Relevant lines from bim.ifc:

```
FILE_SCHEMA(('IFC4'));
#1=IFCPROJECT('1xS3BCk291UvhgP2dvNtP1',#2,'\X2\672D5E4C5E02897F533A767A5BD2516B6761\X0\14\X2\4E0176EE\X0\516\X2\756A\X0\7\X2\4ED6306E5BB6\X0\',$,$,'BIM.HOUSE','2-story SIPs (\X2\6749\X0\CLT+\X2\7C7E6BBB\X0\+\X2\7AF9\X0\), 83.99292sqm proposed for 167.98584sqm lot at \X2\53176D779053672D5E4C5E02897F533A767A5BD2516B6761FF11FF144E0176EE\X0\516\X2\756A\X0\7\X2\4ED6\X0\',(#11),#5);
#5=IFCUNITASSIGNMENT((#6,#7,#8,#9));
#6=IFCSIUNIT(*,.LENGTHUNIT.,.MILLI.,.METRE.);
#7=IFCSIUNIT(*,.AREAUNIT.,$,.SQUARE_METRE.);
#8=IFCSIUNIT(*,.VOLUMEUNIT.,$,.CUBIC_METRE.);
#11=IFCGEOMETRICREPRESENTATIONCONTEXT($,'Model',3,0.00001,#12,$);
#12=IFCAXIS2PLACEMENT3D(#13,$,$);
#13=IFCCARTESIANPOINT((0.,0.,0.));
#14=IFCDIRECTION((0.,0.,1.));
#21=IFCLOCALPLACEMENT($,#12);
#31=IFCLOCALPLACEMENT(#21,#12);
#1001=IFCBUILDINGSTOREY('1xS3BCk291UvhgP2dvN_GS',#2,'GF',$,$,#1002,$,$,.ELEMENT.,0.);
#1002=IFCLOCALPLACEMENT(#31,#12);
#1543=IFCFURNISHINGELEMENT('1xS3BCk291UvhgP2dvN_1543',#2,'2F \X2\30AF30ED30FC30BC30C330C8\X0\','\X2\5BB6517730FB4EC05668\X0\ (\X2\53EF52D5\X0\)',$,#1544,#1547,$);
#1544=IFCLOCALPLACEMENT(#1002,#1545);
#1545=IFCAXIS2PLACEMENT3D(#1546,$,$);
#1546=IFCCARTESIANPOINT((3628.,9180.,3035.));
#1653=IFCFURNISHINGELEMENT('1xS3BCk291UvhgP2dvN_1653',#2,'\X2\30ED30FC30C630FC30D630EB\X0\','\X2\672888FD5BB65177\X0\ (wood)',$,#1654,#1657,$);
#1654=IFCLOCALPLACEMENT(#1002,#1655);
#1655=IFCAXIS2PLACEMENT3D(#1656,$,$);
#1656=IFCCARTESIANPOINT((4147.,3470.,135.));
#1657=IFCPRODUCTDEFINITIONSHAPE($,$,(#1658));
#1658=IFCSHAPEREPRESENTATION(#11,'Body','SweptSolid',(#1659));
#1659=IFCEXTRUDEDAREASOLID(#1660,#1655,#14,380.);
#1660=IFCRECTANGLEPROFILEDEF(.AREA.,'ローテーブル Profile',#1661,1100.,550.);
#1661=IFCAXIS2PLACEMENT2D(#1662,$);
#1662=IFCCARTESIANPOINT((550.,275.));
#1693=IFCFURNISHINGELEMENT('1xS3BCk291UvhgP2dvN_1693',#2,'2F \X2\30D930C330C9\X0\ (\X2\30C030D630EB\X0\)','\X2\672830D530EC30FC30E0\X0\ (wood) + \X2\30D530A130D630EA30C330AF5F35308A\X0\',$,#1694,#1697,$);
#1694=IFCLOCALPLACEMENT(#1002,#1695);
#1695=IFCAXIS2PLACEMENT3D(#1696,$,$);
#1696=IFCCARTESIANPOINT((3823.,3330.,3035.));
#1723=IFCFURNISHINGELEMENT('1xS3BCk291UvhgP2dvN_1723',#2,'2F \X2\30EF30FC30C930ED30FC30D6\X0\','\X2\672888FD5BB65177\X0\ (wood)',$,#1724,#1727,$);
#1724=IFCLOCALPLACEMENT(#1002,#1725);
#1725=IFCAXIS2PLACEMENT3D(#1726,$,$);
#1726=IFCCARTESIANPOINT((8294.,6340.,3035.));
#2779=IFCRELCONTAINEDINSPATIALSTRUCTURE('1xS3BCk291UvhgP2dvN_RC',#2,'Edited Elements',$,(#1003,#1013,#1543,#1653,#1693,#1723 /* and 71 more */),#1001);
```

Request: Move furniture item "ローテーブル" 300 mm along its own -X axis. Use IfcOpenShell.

```python
import ifcopenshell
import ifcopenshell.api.geometry
import ifcopenshell.util.placement
import ifcopenshell.util.unit

model = ifcopenshell.open("bim.ifc")
unit_scale = ifcopenshell.util.unit.calculate_unit_scale(model)

item = model.by_guid("1xS3BCk291UvhgP2dvN_1653")
matrix = ifcopenshell.util.placement.get_local_placement(item.ObjectPlacement)
matrix[:3, 3] -= matrix[:3, 0] * 0.3 / unit_scale
ifcopenshell.api.geometry.edit_object_placement(model, product=item, matrix=matrix, is_si=False)

print(ifcopenshell.util.placement.get_local_placement(item.ObjectPlacement).round(3) + 0.0)

model.write("bim_v2.ifc")
```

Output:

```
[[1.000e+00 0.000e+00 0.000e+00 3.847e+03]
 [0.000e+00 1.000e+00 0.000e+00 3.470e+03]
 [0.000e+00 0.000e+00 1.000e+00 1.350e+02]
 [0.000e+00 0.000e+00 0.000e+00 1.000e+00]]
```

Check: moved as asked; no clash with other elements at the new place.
